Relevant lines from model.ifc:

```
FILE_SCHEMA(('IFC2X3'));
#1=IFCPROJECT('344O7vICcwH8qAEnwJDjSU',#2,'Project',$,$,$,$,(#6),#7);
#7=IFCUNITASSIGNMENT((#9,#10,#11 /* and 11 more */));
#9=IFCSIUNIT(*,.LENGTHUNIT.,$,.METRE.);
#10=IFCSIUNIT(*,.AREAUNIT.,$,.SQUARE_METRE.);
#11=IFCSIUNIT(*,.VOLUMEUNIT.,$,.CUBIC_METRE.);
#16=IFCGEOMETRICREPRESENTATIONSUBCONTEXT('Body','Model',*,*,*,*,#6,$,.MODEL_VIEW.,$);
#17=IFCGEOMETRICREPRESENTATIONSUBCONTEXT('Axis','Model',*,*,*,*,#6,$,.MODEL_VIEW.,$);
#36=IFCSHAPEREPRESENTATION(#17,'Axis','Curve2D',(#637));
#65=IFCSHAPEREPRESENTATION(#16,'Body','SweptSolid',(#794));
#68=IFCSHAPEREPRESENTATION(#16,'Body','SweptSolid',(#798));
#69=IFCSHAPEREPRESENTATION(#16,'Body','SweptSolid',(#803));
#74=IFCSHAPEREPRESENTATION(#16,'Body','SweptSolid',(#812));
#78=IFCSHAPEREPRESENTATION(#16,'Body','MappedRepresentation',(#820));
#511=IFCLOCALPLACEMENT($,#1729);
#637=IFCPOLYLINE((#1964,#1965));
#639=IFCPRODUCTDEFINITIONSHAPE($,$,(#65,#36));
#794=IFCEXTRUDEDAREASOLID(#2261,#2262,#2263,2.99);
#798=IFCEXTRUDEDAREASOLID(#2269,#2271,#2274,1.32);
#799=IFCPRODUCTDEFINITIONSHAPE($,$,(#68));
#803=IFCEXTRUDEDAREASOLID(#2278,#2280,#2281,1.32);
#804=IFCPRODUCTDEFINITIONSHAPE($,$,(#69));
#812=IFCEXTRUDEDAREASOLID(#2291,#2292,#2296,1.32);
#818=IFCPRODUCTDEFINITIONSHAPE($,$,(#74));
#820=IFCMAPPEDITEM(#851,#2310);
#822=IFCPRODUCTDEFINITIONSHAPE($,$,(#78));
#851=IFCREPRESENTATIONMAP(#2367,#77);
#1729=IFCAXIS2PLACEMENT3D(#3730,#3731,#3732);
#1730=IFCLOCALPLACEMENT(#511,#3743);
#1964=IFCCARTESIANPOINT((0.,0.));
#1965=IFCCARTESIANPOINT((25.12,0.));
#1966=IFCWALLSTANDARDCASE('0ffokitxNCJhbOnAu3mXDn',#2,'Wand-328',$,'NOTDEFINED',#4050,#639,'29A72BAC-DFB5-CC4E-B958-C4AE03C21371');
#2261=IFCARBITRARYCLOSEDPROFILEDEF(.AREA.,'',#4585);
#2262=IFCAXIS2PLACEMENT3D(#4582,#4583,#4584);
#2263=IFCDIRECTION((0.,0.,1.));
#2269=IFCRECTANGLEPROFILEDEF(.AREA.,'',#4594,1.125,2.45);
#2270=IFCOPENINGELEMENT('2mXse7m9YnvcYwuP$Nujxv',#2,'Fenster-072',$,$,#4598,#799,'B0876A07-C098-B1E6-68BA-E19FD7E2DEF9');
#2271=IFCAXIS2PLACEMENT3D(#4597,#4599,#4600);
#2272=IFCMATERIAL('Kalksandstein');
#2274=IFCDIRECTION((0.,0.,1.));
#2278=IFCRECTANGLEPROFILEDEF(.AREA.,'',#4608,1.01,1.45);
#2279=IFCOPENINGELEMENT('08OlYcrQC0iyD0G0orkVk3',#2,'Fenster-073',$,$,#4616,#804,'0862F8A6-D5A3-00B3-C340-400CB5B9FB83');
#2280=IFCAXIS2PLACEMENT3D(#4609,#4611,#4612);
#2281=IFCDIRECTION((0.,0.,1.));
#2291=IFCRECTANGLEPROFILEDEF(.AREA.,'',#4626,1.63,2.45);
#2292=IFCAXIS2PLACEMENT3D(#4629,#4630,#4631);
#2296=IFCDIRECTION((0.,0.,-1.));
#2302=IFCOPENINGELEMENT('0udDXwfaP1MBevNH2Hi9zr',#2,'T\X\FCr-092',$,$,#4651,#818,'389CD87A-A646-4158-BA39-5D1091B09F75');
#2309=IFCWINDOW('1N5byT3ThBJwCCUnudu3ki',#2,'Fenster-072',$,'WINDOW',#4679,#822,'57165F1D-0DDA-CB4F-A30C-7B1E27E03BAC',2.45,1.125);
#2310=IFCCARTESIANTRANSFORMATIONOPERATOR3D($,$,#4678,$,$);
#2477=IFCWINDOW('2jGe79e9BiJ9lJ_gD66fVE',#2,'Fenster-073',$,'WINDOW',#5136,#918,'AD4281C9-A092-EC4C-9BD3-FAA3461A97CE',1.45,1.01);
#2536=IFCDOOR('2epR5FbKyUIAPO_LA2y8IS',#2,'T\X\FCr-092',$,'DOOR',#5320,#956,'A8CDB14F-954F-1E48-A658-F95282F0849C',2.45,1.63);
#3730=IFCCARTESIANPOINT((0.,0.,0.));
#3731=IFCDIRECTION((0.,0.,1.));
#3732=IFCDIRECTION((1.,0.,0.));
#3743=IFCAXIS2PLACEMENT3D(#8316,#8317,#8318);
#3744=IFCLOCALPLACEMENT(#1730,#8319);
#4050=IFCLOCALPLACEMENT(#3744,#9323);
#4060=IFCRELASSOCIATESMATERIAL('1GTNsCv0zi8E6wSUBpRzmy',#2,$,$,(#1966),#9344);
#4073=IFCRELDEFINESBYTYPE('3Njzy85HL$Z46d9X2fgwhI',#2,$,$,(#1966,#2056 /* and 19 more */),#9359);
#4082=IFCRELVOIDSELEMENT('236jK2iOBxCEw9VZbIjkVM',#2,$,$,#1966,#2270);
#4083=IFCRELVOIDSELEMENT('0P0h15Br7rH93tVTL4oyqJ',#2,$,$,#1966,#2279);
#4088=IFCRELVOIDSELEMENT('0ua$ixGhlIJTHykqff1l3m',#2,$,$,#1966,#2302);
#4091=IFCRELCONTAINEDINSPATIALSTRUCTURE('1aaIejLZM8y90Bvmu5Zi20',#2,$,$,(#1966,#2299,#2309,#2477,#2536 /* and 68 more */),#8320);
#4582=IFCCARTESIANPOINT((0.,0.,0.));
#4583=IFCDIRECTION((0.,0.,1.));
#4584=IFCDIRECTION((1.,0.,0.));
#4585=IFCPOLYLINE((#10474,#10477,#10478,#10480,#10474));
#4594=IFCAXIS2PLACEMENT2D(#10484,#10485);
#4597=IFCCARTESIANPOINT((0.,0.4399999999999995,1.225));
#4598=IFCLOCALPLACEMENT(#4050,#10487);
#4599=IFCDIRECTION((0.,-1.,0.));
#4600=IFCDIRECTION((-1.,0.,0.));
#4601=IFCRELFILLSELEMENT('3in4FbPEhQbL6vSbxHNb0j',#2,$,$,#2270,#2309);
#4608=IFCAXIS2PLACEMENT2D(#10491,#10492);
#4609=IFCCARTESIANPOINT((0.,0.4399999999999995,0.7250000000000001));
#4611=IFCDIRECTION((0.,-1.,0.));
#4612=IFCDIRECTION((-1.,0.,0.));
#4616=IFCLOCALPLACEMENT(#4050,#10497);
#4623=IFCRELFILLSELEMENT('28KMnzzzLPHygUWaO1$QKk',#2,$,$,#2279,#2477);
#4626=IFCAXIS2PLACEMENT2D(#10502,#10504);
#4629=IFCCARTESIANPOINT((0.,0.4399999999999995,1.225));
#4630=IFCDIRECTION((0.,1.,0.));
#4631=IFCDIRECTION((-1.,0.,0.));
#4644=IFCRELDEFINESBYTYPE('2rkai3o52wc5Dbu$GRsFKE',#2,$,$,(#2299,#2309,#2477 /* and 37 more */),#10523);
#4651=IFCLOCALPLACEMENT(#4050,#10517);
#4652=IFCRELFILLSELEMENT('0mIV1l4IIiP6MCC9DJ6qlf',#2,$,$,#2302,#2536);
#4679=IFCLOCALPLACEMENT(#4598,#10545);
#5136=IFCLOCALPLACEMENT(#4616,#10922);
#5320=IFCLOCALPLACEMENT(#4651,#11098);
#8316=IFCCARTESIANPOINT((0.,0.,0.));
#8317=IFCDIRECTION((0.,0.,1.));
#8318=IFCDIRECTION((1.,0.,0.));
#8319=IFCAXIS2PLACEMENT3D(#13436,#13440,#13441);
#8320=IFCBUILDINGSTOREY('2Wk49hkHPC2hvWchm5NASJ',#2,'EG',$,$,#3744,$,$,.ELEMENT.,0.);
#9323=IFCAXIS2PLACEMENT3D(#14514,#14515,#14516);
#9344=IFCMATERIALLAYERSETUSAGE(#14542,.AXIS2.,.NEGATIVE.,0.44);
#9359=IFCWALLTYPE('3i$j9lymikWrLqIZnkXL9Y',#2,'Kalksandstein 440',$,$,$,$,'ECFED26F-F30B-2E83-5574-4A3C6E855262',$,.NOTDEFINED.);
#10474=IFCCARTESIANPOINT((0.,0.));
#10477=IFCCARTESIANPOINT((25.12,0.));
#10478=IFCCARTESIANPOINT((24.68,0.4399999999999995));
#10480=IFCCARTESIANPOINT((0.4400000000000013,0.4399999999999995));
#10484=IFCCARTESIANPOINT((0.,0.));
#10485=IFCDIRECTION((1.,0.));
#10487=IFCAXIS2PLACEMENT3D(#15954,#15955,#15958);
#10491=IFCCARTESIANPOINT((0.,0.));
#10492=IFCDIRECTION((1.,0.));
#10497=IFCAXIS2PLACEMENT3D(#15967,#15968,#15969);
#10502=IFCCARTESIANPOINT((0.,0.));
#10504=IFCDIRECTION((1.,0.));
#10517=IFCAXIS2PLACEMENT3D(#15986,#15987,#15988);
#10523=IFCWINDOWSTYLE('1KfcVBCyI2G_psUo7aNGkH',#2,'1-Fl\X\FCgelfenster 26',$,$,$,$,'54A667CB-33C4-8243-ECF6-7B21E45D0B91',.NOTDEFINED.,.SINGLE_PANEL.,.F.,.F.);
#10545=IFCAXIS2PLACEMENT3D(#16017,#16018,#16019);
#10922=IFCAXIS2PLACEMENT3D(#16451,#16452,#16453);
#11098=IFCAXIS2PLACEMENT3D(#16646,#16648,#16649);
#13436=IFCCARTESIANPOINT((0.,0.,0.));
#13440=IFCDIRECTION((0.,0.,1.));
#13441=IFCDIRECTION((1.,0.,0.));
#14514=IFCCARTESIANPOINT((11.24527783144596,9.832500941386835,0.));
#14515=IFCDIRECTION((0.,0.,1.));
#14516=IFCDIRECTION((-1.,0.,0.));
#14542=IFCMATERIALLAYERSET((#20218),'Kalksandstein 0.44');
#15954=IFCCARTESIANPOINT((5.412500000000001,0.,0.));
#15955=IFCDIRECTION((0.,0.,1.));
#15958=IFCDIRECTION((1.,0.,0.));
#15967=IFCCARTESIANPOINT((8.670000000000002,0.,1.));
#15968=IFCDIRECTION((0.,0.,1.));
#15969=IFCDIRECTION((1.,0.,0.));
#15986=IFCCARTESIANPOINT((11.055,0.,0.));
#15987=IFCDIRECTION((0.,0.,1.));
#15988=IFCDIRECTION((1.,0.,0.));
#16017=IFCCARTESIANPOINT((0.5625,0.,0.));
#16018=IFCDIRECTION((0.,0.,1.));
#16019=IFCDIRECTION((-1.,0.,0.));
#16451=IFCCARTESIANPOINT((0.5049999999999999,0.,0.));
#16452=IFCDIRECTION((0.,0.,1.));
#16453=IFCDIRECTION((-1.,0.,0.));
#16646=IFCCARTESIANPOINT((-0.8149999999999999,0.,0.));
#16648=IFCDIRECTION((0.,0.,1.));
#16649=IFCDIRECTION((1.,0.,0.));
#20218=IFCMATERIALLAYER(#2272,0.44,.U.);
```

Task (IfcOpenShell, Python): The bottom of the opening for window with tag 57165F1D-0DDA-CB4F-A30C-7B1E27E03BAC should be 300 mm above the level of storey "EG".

```python
import numpy as np
import ifcopenshell
import ifcopenshell.api.geometry
import ifcopenshell.geom
import ifcopenshell.util.element
import ifcopenshell.util.placement
import ifcopenshell.util.shape
import ifcopenshell.util.unit

model = ifcopenshell.open("model.ifc")
unit_scale = ifcopenshell.util.unit.calculate_unit_scale(model)

window = model.by_guid("1N5byT3ThBJwCCUnudu3ki")
opening = window.FillsVoids[0].RelatingOpeningElement
storey = ifcopenshell.util.element.get_container(window, ifc_class="IfcBuildingStorey")
level = ifcopenshell.util.placement.get_local_placement(storey.ObjectPlacement)[2, 3]

# The opening's origin need not be at the sill, so measure its lowest point.
shape = ifcopenshell.geom.create_shape(ifcopenshell.geom.settings(), opening)
bottom = ifcopenshell.util.shape.get_shape_bottom_elevation(shape, shape.geometry) / unit_scale
dz = level + 0.3 / unit_scale - bottom

shift = np.array([0.0, 0.0, dz])
# The window is placed relative to its opening, so it follows when the opening moves.
matrix = ifcopenshell.util.placement.get_local_placement(opening.ObjectPlacement)
matrix[:3, 3] += shift
ifcopenshell.api.geometry.edit_object_placement(
    model, product=opening, matrix=matrix, is_si=False, should_transform_children=True
)

print(f"moved by {dz * unit_scale:+.3f} m")

model.write("model_v2.ifc")
```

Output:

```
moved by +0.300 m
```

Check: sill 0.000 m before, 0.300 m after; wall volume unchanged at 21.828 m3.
